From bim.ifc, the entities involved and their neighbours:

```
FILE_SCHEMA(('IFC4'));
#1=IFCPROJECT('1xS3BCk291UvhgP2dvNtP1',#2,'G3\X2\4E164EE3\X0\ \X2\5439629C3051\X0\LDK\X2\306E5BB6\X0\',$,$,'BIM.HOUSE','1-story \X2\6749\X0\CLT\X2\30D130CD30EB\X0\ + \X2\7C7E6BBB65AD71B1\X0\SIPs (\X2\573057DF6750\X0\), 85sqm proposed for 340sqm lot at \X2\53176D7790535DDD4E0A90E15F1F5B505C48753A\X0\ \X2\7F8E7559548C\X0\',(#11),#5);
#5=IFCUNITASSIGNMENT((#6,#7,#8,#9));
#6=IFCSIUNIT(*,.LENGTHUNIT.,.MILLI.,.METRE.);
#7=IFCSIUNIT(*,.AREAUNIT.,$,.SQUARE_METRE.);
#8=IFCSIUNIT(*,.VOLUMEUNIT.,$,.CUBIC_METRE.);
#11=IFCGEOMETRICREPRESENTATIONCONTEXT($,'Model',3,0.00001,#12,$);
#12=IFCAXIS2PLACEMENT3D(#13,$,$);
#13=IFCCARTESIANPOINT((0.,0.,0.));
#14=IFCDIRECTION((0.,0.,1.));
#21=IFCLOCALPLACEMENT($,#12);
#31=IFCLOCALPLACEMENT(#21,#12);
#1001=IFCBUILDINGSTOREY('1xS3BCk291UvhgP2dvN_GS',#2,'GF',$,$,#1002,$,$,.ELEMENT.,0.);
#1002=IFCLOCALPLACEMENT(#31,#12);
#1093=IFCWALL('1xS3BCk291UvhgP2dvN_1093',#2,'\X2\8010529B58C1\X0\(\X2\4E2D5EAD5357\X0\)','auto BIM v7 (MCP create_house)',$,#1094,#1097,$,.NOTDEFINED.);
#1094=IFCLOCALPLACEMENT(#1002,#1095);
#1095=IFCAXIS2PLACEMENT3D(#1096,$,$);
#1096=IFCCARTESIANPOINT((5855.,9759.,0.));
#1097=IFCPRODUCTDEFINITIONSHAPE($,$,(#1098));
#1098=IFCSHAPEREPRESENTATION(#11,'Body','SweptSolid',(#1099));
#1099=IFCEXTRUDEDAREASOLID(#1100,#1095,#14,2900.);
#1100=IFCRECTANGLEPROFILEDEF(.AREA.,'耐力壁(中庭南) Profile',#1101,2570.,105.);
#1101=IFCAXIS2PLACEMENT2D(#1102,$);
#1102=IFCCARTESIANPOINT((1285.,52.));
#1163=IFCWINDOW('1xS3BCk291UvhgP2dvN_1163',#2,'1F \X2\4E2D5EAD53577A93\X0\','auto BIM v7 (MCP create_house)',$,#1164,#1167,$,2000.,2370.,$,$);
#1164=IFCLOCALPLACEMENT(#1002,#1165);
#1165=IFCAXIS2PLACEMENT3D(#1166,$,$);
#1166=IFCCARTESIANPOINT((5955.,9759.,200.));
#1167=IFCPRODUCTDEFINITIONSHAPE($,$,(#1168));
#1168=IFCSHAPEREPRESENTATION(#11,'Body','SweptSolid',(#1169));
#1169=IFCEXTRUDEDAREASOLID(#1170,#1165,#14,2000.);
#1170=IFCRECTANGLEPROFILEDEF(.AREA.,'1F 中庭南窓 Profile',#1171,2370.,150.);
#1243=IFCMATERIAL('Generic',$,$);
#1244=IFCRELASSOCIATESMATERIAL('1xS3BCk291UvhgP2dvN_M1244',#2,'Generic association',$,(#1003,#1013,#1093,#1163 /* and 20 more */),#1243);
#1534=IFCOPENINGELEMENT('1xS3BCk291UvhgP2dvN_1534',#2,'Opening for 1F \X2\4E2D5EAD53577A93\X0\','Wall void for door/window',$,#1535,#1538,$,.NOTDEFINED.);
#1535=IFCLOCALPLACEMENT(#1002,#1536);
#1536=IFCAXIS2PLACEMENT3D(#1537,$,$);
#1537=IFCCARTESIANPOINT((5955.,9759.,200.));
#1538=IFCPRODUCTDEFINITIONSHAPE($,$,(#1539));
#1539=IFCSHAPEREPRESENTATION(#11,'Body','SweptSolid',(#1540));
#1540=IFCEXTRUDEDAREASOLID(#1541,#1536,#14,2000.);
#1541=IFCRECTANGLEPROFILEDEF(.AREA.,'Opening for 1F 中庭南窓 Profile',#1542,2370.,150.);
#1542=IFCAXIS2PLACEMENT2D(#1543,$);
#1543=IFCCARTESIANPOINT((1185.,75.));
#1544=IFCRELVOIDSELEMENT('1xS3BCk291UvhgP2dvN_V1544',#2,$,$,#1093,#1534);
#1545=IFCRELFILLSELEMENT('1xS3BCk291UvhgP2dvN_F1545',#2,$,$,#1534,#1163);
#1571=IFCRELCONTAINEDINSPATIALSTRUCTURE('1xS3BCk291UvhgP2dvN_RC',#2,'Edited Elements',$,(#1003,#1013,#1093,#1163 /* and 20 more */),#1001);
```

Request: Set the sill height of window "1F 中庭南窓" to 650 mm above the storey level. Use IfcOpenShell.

```python
import numpy as np
import ifcopenshell
import ifcopenshell.api.geometry
import ifcopenshell.geom
import ifcopenshell.util.element
import ifcopenshell.util.placement
import ifcopenshell.util.shape
import ifcopenshell.util.unit

model = ifcopenshell.open("bim.ifc")
unit_scale = ifcopenshell.util.unit.calculate_unit_scale(model)

window = model.by_guid("1xS3BCk291UvhgP2dvN_1163")
opening = window.FillsVoids[0].RelatingOpeningElement
storey = ifcopenshell.util.element.get_container(window, ifc_class="IfcBuildingStorey")
level = ifcopenshell.util.placement.get_local_placement(storey.ObjectPlacement)[2, 3]

# The opening's origin need not be at the sill, so measure its lowest point.
shape = ifcopenshell.geom.create_shape(ifcopenshell.geom.settings(), opening)
bottom = ifcopenshell.util.shape.get_shape_bottom_elevation(shape, shape.geometry) / unit_scale
dz = level + 650.0 - bottom

shift = np.array([0.0, 0.0, dz])
# The window is not placed relative to its opening, so move both.
for product in (opening, window):
    matrix = ifcopenshell.util.placement.get_local_placement(product.ObjectPlacement)
    matrix[:3, 3] += shift
    ifcopenshell.api.geometry.edit_object_placement(model, product=product, matrix=matrix, is_si=False)

print(f"moved by {dz * unit_scale:+.3f} m")

model.write("bim_rev.ifc")
```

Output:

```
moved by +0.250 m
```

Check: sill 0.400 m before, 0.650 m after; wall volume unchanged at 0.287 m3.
